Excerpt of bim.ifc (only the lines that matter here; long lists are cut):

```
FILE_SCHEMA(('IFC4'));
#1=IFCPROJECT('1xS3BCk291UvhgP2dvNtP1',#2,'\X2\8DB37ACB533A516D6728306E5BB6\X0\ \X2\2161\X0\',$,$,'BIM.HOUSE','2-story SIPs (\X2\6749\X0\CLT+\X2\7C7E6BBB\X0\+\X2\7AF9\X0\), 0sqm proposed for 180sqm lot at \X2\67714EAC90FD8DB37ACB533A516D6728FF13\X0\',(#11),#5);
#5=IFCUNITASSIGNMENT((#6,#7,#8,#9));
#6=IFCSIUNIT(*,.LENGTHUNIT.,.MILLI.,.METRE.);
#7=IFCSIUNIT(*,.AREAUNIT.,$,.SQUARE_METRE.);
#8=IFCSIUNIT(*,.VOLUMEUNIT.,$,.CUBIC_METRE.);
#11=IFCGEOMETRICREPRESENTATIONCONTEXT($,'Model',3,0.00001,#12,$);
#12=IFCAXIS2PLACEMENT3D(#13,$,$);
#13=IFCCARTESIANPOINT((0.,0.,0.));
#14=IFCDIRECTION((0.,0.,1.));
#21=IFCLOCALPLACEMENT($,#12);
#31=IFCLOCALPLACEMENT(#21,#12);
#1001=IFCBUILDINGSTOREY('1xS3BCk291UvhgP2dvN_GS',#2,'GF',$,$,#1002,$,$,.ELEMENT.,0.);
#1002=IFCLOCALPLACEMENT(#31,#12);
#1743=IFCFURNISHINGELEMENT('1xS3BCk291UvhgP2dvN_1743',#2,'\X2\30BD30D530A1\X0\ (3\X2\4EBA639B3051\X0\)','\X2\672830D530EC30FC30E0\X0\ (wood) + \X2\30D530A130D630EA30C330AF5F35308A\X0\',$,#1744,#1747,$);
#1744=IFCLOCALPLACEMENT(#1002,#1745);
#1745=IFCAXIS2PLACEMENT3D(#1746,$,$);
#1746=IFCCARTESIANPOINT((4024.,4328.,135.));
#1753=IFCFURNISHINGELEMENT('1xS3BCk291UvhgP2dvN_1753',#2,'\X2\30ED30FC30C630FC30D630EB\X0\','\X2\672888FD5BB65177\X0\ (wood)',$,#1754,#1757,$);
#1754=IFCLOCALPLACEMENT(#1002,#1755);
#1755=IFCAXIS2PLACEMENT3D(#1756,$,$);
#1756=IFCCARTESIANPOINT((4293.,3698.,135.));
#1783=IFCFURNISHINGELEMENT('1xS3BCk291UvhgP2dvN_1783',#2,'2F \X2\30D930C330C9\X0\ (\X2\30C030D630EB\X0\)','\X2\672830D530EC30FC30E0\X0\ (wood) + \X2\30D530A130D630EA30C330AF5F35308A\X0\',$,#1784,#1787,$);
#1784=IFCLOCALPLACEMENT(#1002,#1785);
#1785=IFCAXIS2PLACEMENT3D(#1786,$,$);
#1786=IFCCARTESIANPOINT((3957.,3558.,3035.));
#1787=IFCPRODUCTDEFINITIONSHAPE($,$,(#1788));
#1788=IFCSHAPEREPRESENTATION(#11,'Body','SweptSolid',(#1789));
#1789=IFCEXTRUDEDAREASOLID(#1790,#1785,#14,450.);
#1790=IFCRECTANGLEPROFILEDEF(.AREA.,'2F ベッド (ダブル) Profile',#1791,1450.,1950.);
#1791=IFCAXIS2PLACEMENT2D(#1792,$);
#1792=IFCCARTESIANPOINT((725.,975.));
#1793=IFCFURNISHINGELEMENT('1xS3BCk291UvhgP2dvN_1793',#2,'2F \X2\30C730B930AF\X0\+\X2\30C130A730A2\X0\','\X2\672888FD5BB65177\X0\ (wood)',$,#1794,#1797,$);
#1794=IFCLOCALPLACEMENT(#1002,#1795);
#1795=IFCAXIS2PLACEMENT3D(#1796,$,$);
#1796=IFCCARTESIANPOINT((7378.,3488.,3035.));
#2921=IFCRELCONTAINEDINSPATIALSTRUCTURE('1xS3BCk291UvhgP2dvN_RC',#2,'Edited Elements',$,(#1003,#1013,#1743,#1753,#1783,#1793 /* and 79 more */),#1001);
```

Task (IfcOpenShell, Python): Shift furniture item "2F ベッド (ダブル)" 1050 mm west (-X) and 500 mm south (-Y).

```python
import ifcopenshell
import ifcopenshell.api.geometry
import ifcopenshell.util.placement

model = ifcopenshell.open("bim.ifc")

item = model.by_guid("1xS3BCk291UvhgP2dvN_1783")
matrix = ifcopenshell.util.placement.get_local_placement(item.ObjectPlacement)
matrix[0, 3] -= 1050.0
matrix[1, 3] -= 500.0
ifcopenshell.api.geometry.edit_object_placement(model, product=item, matrix=matrix, is_si=False)

print(ifcopenshell.util.placement.get_local_placement(item.ObjectPlacement).round(3) + 0.0)

model.write("bim-out.ifc")
```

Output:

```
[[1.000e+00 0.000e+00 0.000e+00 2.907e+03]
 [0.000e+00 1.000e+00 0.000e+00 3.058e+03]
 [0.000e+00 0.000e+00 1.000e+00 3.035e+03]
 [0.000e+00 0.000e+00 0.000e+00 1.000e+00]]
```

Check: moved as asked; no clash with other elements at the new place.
